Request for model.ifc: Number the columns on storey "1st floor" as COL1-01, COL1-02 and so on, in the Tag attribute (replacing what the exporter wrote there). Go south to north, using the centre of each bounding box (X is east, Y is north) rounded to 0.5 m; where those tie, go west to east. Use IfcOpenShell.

First a look at what the model holds.

```python
import ifcopenshell
import ifcopenshell.util.element
import ifcopenshell.util.placement

model = ifcopenshell.open("model.ifc")
print(model.schema)
storey = next(s for s in model.by_type("IfcBuildingStorey") if s.Name == "1st floor")
columns = [e for e in ifcopenshell.util.element.get_decomposition(storey) if e.is_a("IfcColumn")]
for e in sorted(columns, key=lambda e: e.id()):
    origin = ifcopenshell.util.placement.get_local_placement(e.ObjectPlacement)[:3, 3]
    print(e.id(), e.Tag, e.Name, origin.round(2) + 0.0, sep=" | ")
```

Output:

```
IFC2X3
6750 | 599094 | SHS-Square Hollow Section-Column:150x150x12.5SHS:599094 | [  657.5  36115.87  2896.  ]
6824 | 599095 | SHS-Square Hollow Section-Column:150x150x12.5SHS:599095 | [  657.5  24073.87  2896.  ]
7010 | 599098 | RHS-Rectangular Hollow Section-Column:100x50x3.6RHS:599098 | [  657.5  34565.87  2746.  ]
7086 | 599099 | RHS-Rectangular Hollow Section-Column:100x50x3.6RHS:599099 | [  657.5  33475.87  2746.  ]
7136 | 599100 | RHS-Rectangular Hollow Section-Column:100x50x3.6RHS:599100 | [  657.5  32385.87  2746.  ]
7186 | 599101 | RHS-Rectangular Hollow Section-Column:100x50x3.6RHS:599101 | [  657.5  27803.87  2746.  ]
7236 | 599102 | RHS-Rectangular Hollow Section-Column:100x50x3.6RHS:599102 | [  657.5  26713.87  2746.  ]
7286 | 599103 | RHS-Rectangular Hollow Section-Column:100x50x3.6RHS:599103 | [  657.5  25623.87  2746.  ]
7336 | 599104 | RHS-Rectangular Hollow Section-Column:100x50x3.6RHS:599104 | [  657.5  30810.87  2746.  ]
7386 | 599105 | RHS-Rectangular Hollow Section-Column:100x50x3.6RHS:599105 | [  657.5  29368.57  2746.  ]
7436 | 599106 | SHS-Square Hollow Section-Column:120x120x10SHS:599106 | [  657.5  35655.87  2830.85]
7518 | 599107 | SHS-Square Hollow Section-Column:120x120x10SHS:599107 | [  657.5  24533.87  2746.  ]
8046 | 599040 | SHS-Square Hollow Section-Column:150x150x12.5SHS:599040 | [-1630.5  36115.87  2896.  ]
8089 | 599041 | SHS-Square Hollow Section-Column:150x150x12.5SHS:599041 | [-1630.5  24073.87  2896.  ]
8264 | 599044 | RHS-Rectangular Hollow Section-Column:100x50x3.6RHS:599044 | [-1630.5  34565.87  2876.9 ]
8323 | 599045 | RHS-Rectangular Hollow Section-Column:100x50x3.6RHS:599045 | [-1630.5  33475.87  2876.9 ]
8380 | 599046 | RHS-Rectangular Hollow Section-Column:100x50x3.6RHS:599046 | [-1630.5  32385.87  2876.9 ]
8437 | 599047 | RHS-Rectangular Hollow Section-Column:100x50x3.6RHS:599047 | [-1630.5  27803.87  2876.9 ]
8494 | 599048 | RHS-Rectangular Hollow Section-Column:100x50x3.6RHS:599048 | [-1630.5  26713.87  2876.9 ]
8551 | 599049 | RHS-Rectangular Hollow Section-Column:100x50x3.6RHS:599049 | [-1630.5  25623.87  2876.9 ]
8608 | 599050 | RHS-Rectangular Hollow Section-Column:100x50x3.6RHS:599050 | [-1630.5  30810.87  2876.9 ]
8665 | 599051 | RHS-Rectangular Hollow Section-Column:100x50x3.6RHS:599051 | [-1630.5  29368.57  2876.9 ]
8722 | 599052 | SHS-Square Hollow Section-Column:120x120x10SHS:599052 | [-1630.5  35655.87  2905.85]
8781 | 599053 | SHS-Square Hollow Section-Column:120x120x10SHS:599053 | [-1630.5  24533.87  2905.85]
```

```python
import ifcopenshell
import ifcopenshell.geom
import ifcopenshell.util.element
import ifcopenshell.util.shape

model = ifcopenshell.open("model.ifc")
settings = ifcopenshell.geom.settings()
settings.set("use-world-coords", True)


def centre(element):
    shape = ifcopenshell.geom.create_shape(settings, element)
    return ifcopenshell.util.shape.get_bbox_centroid(shape.geometry)


storey = next(s for s in model.by_type("IfcBuildingStorey") if s.Name == "1st floor")
columns = [e for e in ifcopenshell.util.element.get_decomposition(storey) if e.is_a("IfcColumn")]

# Insertion points can sit at a corner or the storey origin, so sort by the geometry (in metres).
centres = {e: centre(e) for e in columns}
columns.sort(key=lambda e: (round(centres[e][1] / 0.5), centres[e][0]))

for i, e in enumerate(columns, start=1):
    number = f"COL1-{i:02d}"
    e.Tag = number
    print(e.id(), number)

model.write("model_edited.ifc")
```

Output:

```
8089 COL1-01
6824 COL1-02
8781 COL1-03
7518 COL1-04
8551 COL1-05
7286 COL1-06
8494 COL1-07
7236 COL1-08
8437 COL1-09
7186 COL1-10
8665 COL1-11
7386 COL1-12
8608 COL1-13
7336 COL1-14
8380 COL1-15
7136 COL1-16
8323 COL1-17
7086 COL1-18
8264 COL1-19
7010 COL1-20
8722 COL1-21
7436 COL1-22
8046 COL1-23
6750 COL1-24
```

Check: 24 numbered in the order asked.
